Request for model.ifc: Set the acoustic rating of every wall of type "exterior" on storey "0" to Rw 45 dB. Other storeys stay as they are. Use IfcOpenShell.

First a look at what the model holds.

```python
import ifcopenshell
import ifcopenshell.util.element

model = ifcopenshell.open("model.ifc")
print(model.schema)
storey = next(s for s in model.by_type("IfcBuildingStorey") if s.Name == "0")
walls = [e for e in ifcopenshell.util.element.get_decomposition(storey) if e.is_a("IfcWall")]
seen = {}
for e in walls:
    element_type = ifcopenshell.util.element.get_type(e)
    key = (element_type.Name if element_type != e and element_type else None, ifcopenshell.util.element.get_pset(e, "Pset_WallCommon", "AcousticRating"))
    seen[key] = seen.get(key, 0) + 1
for (name, value), count in sorted(seen.items(), key=str):
    print(count, "x", name, "|", value)
```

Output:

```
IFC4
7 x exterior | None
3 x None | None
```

```python
import ifcopenshell
import ifcopenshell.api.pset
import ifcopenshell.util.element

model = ifcopenshell.open("model.ifc")

storey = next(s for s in model.by_type("IfcBuildingStorey") if s.Name == "0")
walls = [e for e in ifcopenshell.util.element.get_decomposition(storey) if e.is_a("IfcWall")]

count = 0
for e in walls:
    element_type = ifcopenshell.util.element.get_type(e)
    if element_type in (None, e) or element_type.Name != "exterior":
        continue
    # add_pset returns the element's existing set when there is one.
    pset = ifcopenshell.api.pset.add_pset(model, product=e, name="Pset_WallCommon")
    ifcopenshell.api.pset.edit_pset(model, pset=pset, properties={"AcousticRating": "Rw 45 dB"})
    count += 1

print(count, "walls updated")

model.write("model_edited.ifc")
```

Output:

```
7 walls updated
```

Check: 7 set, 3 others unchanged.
